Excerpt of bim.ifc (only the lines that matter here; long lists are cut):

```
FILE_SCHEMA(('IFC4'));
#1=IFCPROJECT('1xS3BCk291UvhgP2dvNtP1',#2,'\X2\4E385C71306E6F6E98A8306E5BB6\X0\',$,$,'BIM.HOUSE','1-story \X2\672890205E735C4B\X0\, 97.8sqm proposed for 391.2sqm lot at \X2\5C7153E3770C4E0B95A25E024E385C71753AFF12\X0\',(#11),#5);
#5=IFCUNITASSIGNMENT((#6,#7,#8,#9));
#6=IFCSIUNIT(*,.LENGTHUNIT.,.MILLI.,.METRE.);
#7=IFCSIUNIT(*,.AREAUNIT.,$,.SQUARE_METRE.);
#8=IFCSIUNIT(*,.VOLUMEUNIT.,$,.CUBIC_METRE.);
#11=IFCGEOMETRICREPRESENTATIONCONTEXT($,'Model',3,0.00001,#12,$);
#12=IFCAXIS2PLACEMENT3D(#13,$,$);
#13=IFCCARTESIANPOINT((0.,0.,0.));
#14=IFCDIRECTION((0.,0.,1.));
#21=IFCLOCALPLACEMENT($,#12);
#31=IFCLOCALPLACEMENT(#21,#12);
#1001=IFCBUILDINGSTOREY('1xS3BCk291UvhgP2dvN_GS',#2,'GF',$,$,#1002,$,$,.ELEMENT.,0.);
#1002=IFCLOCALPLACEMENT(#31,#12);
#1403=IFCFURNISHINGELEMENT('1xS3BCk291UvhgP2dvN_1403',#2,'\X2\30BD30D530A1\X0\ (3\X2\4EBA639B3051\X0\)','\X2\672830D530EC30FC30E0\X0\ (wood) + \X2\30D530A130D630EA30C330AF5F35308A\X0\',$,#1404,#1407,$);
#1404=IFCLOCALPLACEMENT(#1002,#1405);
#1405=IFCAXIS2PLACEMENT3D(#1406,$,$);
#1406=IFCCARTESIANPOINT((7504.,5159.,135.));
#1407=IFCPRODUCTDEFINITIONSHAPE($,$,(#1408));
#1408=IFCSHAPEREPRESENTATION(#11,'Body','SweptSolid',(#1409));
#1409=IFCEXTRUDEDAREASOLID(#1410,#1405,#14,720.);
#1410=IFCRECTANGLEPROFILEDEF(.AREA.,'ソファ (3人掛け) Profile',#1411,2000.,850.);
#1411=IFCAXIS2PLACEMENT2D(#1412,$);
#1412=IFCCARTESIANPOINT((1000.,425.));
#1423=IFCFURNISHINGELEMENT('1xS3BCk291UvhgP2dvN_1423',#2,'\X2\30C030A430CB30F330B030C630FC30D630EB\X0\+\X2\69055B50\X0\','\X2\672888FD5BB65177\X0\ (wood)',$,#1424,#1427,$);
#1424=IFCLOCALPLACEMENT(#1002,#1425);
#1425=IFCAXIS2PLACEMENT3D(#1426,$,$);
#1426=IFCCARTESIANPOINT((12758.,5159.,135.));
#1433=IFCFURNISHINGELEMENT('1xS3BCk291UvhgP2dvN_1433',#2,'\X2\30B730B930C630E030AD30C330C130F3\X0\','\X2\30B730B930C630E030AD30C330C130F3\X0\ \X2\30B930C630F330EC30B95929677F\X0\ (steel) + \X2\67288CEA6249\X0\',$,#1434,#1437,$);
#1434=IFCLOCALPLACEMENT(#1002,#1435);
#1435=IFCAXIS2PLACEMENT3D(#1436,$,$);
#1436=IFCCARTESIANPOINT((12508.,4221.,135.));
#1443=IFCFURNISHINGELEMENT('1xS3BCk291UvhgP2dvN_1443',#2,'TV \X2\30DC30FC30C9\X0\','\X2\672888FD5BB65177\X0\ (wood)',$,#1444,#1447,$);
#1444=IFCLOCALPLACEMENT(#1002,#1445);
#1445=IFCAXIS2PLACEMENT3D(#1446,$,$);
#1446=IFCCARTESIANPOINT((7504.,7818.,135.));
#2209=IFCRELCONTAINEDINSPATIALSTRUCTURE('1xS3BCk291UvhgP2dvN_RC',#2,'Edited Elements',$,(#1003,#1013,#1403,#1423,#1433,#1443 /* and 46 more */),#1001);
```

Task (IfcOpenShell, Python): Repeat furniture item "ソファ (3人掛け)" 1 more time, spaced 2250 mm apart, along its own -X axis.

```python
import ifcopenshell
import ifcopenshell.api.geometry
import ifcopenshell.api.root
import ifcopenshell.util.element
import ifcopenshell.util.placement

model = ifcopenshell.open("bim.ifc")


def reuse_history(source, copy):
    """copy_class also copies each property set's owner history, people and application; keep the originals."""
    for rel in copy.IsDefinedBy:
        if rel.is_a("IfcRelDefinesByProperties") and (history := rel.RelatingPropertyDefinition.OwnerHistory):
            rel.RelatingPropertyDefinition.OwnerHistory = source.OwnerHistory
            ifcopenshell.util.element.remove_deep2(model, history)


source = model.by_guid("1xS3BCk291UvhgP2dvN_1403")
base = ifcopenshell.util.placement.get_local_placement(source.ObjectPlacement)
step = -base[:3, 0] * 2250.0

for i in range(1, 2):
    copy = ifcopenshell.api.root.copy_class(model, product=source)
    copy.Representation = ifcopenshell.util.element.copy_deep(
        model, source.Representation, exclude=["IfcGeometricRepresentationContext", "IfcRepresentationMap"]
    )
    reuse_history(source, copy)
    matrix = base.copy()
    matrix[:3, 3] += i * step
    print("added at", matrix[:3, 3].round(3) + 0.0)
    ifcopenshell.api.geometry.edit_object_placement(model, product=copy, matrix=matrix, is_si=False)

model.write("bim-out.ifc")
```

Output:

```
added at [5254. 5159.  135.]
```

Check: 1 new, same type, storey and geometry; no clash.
